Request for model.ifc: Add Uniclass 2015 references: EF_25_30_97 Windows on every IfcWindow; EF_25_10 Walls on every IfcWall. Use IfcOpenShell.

First a look at what the model holds.

```python
import ifcopenshell

model = ifcopenshell.open("model.ifc")
print(model.schema)
print("classifications:", [c.Name for c in model.by_type("IfcClassification")])
for ifc_class in ("IfcDoor", "IfcRoof", "IfcStair", "IfcWall", "IfcWindow"):
    print(ifc_class, len(model.by_type(ifc_class)))
```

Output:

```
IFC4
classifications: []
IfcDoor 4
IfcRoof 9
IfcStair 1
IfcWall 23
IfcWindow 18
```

```python
import ifcopenshell
import ifcopenshell.api.classification

model = ifcopenshell.open("model.ifc")

system = ifcopenshell.api.classification.add_classification(model, classification="Uniclass 2015")

codes = {
    "IfcWindow": ("EF_25_30_97", "Windows"),
    "IfcWall": ("EF_25_10", "Walls"),
}
for ifc_class, (code, name) in codes.items():
    products = model.by_type(ifc_class)
    ifcopenshell.api.classification.add_reference(
        model, products=products, classification=system, identification=code, name=name
    )
    print(code, len(products))

model.write("model-out.ifc")
```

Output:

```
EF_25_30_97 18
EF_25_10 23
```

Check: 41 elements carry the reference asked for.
